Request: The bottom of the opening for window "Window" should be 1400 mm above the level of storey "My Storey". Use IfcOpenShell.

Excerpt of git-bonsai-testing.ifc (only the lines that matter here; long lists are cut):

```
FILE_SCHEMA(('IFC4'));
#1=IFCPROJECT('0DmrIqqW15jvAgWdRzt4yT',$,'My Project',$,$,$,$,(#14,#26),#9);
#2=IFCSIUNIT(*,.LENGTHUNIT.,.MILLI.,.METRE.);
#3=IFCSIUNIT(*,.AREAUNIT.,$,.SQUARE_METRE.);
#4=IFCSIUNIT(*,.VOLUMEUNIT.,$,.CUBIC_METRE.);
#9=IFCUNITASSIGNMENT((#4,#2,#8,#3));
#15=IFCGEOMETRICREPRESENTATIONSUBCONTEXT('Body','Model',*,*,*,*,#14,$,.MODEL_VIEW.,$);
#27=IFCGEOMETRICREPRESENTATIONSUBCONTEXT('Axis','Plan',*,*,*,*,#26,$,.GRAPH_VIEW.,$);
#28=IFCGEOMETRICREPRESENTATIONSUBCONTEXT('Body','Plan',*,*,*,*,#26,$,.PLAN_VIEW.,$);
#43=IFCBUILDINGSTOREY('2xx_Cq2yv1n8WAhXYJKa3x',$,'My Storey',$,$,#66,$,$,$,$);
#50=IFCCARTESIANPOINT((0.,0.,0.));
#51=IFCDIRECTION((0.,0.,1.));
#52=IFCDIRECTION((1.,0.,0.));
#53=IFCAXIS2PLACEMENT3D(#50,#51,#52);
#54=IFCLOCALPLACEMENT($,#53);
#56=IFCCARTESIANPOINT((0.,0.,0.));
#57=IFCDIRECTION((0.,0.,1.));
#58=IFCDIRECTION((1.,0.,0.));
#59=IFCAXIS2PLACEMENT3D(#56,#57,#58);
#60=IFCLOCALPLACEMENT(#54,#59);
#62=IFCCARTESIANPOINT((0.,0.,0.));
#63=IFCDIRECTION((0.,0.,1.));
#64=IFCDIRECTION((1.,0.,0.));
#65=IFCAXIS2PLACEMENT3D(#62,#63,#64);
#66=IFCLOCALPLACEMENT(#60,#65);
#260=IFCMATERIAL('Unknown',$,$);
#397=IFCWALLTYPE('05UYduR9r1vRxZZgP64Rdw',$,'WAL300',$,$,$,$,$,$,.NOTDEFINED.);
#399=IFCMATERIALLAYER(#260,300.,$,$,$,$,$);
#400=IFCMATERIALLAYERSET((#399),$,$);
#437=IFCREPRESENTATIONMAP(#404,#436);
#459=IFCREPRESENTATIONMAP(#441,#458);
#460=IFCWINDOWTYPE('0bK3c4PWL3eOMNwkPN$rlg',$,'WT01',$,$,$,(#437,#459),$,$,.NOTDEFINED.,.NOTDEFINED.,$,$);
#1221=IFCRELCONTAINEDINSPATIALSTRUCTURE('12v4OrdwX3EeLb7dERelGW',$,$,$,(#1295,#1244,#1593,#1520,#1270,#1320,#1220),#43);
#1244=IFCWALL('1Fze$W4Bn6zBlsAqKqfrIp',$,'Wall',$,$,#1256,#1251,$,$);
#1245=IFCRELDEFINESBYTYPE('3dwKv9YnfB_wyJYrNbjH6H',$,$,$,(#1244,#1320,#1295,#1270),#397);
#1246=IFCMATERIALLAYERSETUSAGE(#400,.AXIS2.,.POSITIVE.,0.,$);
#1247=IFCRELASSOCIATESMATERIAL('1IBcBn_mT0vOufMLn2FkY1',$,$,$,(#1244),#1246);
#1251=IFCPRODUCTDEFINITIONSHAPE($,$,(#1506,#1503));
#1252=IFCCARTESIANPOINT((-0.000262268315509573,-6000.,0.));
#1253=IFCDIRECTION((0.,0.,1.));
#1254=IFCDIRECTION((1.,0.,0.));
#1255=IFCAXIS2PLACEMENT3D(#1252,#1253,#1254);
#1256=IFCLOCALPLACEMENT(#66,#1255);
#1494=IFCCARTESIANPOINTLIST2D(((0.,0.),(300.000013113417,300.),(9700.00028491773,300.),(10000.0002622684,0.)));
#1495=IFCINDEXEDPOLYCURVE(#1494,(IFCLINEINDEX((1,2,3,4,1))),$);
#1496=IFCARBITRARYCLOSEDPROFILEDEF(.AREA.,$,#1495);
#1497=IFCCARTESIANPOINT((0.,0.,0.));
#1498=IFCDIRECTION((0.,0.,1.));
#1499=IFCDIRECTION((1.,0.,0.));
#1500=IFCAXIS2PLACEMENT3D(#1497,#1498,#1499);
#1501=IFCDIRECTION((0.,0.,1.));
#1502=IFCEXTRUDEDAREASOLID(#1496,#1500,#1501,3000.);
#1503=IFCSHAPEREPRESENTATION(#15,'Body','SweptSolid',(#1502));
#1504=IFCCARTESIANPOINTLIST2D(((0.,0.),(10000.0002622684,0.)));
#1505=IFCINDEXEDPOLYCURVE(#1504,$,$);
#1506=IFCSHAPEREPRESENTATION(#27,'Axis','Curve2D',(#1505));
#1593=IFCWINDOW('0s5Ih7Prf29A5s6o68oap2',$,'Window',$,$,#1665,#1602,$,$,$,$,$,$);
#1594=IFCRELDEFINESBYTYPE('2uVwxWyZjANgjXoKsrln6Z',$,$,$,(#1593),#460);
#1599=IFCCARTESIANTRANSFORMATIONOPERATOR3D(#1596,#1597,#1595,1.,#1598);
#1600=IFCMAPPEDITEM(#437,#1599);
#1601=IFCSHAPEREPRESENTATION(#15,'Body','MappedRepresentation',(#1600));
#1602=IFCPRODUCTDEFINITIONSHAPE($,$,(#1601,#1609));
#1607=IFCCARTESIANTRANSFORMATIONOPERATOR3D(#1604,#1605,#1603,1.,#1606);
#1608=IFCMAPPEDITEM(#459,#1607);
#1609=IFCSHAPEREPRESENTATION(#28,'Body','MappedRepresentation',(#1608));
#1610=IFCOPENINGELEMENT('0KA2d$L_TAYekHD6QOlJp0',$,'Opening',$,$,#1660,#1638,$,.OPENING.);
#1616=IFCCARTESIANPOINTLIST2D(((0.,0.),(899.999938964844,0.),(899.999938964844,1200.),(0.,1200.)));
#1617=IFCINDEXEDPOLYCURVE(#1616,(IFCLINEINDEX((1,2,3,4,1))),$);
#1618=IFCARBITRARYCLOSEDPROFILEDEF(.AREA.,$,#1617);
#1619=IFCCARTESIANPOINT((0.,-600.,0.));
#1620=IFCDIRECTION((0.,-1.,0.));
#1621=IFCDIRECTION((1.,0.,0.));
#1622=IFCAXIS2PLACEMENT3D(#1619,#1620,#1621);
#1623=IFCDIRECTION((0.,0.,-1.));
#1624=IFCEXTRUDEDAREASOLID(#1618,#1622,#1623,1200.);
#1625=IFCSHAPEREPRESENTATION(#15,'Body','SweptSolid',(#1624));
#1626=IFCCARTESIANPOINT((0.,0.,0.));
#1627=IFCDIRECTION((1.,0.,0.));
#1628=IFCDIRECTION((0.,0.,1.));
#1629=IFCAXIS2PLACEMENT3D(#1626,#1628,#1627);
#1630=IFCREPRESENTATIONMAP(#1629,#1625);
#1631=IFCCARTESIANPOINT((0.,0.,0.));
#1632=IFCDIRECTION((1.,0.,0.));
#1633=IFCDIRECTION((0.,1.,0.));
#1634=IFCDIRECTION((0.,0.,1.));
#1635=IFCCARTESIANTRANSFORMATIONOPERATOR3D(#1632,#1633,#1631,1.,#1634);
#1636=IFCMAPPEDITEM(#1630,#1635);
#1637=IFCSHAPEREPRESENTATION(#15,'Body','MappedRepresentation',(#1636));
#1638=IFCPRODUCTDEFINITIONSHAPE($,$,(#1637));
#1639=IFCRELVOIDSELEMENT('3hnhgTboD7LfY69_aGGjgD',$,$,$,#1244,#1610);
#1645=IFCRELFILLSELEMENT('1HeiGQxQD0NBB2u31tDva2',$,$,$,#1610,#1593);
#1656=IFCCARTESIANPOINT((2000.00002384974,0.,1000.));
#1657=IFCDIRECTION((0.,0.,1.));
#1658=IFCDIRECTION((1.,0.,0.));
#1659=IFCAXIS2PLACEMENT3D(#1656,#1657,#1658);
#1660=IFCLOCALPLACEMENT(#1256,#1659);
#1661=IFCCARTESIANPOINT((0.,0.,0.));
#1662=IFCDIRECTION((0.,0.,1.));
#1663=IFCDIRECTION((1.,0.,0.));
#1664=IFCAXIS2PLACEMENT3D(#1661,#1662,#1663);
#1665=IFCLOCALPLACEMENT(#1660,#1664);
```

```python
import numpy as np
import ifcopenshell
import ifcopenshell.api.geometry
import ifcopenshell.geom
import ifcopenshell.util.element
import ifcopenshell.util.placement
import ifcopenshell.util.shape
import ifcopenshell.util.unit

model = ifcopenshell.open("git-bonsai-testing.ifc")
unit_scale = ifcopenshell.util.unit.calculate_unit_scale(model)

window = model.by_guid("0s5Ih7Prf29A5s6o68oap2")
opening = window.FillsVoids[0].RelatingOpeningElement
storey = ifcopenshell.util.element.get_container(window, ifc_class="IfcBuildingStorey")
level = ifcopenshell.util.placement.get_local_placement(storey.ObjectPlacement)[2, 3]

# The opening's origin need not be at the sill, so measure its lowest point.
shape = ifcopenshell.geom.create_shape(ifcopenshell.geom.settings(), opening)
bottom = ifcopenshell.util.shape.get_shape_bottom_elevation(shape, shape.geometry) / unit_scale
dz = level + 1.4 / unit_scale - bottom

shift = np.array([0.0, 0.0, dz])
# The window is placed relative to its opening, so it follows when the opening moves.
matrix = ifcopenshell.util.placement.get_local_placement(opening.ObjectPlacement)
matrix[:3, 3] += shift
ifcopenshell.api.geometry.edit_object_placement(
    model, product=opening, matrix=matrix, is_si=False, should_transform_children=True
)

print(f"moved by {dz * unit_scale:+.3f} m")

model.write("git-bonsai-testing_v2.ifc")
```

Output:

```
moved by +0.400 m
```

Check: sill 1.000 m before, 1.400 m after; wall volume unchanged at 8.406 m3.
